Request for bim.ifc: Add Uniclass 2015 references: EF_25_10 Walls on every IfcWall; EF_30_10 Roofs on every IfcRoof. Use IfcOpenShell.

First a look at what the model holds.

```python
import ifcopenshell

model = ifcopenshell.open("bim.ifc")
print(model.schema)
print("classifications:", [c.Name for c in model.by_type("IfcClassification")])
for ifc_class in ("IfcDoor", "IfcRoof", "IfcStair", "IfcWall", "IfcWindow"):
    print(ifc_class, len(model.by_type(ifc_class)))
```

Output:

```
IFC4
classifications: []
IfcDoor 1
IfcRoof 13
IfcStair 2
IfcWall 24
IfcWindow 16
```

```python
import ifcopenshell
import ifcopenshell.api.classification

model = ifcopenshell.open("bim.ifc")

system = ifcopenshell.api.classification.add_classification(model, classification="Uniclass 2015")

codes = {
    "IfcWall": ("EF_25_10", "Walls"),
    "IfcRoof": ("EF_30_10", "Roofs"),
}
for ifc_class, (code, name) in codes.items():
    products = model.by_type(ifc_class)
    ifcopenshell.api.classification.add_reference(
        model, products=products, classification=system, identification=code, name=name
    )
    print(code, len(products))

model.write("bim_v2.ifc")
```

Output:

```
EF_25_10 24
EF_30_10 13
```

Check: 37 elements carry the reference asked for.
